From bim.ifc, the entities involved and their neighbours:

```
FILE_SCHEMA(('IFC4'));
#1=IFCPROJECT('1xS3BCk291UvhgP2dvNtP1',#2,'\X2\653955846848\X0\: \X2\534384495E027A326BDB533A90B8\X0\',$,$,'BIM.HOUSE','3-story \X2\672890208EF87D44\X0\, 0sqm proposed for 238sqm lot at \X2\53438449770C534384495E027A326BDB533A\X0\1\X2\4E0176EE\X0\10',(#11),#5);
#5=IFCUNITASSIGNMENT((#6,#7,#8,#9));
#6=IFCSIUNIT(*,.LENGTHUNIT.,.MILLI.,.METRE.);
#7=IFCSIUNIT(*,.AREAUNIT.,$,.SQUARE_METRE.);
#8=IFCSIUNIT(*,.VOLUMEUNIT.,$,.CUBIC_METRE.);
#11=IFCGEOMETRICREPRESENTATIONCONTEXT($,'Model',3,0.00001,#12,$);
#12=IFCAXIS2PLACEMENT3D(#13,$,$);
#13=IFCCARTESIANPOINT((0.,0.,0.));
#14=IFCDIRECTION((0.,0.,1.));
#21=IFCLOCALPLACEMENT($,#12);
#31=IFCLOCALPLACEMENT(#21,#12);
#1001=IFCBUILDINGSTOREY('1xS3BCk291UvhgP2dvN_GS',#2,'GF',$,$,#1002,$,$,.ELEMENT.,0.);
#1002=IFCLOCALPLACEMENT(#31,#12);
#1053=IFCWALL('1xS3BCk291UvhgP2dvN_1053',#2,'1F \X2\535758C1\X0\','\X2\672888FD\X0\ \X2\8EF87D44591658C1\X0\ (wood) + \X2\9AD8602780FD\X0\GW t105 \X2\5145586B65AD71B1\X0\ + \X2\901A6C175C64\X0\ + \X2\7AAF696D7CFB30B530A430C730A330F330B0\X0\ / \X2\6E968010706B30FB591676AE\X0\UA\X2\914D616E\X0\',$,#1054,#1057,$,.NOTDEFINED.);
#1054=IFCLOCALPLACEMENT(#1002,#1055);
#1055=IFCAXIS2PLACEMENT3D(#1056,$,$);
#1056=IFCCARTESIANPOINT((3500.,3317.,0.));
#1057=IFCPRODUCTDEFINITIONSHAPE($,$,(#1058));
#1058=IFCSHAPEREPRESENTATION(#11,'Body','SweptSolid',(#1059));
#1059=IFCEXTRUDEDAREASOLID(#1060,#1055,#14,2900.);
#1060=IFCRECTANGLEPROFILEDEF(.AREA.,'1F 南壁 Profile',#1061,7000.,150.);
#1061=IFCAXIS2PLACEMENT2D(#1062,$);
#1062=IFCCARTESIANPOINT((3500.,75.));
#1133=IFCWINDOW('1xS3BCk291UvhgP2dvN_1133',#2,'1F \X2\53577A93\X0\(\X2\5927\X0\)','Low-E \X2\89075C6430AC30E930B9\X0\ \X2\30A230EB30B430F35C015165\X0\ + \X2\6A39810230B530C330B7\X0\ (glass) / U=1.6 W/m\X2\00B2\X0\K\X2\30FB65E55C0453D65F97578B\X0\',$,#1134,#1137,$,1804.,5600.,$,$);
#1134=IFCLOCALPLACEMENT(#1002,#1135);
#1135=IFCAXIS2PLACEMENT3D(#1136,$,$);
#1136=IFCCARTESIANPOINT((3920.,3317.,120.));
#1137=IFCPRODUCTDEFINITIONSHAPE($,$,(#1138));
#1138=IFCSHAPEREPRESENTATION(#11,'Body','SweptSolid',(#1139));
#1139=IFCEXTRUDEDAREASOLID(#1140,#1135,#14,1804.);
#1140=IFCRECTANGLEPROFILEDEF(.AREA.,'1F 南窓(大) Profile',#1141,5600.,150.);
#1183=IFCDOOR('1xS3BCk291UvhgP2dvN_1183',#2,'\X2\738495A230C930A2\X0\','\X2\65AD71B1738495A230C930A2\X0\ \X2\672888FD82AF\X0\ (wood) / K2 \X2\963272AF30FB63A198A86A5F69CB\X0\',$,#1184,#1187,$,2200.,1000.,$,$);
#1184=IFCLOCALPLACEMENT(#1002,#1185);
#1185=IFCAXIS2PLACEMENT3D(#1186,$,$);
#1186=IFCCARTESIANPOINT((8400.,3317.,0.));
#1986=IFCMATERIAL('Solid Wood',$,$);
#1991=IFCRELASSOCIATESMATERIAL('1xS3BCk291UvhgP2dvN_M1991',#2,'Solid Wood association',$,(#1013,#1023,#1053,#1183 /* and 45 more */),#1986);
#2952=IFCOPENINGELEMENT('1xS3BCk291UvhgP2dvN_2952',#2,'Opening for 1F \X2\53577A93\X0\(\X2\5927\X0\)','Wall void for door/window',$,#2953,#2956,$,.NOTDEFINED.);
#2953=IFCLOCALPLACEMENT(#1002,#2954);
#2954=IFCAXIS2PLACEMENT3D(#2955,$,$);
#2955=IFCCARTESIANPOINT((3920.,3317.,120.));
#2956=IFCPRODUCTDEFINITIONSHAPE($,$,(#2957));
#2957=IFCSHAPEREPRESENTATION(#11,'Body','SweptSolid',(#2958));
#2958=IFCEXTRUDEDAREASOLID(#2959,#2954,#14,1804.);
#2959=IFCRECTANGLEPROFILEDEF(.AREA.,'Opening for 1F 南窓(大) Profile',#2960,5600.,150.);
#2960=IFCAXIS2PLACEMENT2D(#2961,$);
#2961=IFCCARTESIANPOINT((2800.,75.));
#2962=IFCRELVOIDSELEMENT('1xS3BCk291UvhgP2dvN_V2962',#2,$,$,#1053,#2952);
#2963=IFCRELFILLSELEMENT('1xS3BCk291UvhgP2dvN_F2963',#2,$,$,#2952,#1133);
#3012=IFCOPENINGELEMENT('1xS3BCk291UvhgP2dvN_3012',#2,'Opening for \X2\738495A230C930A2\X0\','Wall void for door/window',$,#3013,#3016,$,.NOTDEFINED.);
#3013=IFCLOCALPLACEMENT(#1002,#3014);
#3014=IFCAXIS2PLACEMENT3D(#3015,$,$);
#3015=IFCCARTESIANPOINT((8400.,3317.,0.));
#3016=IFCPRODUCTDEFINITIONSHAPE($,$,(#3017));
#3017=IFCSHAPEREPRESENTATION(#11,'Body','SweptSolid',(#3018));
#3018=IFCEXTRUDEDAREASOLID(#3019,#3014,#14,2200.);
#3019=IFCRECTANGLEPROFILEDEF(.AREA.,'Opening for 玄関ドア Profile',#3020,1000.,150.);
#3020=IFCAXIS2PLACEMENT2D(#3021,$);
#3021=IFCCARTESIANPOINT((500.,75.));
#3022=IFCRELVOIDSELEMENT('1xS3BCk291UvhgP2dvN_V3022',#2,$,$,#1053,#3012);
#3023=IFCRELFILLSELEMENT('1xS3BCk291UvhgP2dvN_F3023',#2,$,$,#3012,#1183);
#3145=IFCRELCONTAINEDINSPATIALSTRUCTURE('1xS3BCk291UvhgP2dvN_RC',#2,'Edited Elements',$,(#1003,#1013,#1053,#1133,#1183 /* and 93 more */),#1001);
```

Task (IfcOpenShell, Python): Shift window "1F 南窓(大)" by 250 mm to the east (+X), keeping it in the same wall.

```python
import ifcopenshell
import ifcopenshell.api.geometry
import ifcopenshell.util.placement
import ifcopenshell.util.unit

model = ifcopenshell.open("bim.ifc")
unit_scale = ifcopenshell.util.unit.calculate_unit_scale(model)

window = model.by_guid("1xS3BCk291UvhgP2dvN_1133")
opening = window.FillsVoids[0].RelatingOpeningElement
wall = opening.VoidsElements[0].RelatingBuildingElement

wall_matrix = ifcopenshell.util.placement.get_local_placement(wall.ObjectPlacement)
shift = wall_matrix[:3, 0] * 0.25 / unit_scale
before = ifcopenshell.util.placement.get_local_placement(window.ObjectPlacement)[:3, 3].copy()

# The window is not placed relative to its opening, so move both.
for product in (opening, window):
    matrix = ifcopenshell.util.placement.get_local_placement(product.ObjectPlacement)
    matrix[:3, 3] += shift
    ifcopenshell.api.geometry.edit_object_placement(model, product=product, matrix=matrix, is_si=False)

after = ifcopenshell.util.placement.get_local_placement(window.ObjectPlacement)[:3, 3]
print("window moved by", (after - before).round(3) + 0.0)

model.write("bim_updated.ifc")
```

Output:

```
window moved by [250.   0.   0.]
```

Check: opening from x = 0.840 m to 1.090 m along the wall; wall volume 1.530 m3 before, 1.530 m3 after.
